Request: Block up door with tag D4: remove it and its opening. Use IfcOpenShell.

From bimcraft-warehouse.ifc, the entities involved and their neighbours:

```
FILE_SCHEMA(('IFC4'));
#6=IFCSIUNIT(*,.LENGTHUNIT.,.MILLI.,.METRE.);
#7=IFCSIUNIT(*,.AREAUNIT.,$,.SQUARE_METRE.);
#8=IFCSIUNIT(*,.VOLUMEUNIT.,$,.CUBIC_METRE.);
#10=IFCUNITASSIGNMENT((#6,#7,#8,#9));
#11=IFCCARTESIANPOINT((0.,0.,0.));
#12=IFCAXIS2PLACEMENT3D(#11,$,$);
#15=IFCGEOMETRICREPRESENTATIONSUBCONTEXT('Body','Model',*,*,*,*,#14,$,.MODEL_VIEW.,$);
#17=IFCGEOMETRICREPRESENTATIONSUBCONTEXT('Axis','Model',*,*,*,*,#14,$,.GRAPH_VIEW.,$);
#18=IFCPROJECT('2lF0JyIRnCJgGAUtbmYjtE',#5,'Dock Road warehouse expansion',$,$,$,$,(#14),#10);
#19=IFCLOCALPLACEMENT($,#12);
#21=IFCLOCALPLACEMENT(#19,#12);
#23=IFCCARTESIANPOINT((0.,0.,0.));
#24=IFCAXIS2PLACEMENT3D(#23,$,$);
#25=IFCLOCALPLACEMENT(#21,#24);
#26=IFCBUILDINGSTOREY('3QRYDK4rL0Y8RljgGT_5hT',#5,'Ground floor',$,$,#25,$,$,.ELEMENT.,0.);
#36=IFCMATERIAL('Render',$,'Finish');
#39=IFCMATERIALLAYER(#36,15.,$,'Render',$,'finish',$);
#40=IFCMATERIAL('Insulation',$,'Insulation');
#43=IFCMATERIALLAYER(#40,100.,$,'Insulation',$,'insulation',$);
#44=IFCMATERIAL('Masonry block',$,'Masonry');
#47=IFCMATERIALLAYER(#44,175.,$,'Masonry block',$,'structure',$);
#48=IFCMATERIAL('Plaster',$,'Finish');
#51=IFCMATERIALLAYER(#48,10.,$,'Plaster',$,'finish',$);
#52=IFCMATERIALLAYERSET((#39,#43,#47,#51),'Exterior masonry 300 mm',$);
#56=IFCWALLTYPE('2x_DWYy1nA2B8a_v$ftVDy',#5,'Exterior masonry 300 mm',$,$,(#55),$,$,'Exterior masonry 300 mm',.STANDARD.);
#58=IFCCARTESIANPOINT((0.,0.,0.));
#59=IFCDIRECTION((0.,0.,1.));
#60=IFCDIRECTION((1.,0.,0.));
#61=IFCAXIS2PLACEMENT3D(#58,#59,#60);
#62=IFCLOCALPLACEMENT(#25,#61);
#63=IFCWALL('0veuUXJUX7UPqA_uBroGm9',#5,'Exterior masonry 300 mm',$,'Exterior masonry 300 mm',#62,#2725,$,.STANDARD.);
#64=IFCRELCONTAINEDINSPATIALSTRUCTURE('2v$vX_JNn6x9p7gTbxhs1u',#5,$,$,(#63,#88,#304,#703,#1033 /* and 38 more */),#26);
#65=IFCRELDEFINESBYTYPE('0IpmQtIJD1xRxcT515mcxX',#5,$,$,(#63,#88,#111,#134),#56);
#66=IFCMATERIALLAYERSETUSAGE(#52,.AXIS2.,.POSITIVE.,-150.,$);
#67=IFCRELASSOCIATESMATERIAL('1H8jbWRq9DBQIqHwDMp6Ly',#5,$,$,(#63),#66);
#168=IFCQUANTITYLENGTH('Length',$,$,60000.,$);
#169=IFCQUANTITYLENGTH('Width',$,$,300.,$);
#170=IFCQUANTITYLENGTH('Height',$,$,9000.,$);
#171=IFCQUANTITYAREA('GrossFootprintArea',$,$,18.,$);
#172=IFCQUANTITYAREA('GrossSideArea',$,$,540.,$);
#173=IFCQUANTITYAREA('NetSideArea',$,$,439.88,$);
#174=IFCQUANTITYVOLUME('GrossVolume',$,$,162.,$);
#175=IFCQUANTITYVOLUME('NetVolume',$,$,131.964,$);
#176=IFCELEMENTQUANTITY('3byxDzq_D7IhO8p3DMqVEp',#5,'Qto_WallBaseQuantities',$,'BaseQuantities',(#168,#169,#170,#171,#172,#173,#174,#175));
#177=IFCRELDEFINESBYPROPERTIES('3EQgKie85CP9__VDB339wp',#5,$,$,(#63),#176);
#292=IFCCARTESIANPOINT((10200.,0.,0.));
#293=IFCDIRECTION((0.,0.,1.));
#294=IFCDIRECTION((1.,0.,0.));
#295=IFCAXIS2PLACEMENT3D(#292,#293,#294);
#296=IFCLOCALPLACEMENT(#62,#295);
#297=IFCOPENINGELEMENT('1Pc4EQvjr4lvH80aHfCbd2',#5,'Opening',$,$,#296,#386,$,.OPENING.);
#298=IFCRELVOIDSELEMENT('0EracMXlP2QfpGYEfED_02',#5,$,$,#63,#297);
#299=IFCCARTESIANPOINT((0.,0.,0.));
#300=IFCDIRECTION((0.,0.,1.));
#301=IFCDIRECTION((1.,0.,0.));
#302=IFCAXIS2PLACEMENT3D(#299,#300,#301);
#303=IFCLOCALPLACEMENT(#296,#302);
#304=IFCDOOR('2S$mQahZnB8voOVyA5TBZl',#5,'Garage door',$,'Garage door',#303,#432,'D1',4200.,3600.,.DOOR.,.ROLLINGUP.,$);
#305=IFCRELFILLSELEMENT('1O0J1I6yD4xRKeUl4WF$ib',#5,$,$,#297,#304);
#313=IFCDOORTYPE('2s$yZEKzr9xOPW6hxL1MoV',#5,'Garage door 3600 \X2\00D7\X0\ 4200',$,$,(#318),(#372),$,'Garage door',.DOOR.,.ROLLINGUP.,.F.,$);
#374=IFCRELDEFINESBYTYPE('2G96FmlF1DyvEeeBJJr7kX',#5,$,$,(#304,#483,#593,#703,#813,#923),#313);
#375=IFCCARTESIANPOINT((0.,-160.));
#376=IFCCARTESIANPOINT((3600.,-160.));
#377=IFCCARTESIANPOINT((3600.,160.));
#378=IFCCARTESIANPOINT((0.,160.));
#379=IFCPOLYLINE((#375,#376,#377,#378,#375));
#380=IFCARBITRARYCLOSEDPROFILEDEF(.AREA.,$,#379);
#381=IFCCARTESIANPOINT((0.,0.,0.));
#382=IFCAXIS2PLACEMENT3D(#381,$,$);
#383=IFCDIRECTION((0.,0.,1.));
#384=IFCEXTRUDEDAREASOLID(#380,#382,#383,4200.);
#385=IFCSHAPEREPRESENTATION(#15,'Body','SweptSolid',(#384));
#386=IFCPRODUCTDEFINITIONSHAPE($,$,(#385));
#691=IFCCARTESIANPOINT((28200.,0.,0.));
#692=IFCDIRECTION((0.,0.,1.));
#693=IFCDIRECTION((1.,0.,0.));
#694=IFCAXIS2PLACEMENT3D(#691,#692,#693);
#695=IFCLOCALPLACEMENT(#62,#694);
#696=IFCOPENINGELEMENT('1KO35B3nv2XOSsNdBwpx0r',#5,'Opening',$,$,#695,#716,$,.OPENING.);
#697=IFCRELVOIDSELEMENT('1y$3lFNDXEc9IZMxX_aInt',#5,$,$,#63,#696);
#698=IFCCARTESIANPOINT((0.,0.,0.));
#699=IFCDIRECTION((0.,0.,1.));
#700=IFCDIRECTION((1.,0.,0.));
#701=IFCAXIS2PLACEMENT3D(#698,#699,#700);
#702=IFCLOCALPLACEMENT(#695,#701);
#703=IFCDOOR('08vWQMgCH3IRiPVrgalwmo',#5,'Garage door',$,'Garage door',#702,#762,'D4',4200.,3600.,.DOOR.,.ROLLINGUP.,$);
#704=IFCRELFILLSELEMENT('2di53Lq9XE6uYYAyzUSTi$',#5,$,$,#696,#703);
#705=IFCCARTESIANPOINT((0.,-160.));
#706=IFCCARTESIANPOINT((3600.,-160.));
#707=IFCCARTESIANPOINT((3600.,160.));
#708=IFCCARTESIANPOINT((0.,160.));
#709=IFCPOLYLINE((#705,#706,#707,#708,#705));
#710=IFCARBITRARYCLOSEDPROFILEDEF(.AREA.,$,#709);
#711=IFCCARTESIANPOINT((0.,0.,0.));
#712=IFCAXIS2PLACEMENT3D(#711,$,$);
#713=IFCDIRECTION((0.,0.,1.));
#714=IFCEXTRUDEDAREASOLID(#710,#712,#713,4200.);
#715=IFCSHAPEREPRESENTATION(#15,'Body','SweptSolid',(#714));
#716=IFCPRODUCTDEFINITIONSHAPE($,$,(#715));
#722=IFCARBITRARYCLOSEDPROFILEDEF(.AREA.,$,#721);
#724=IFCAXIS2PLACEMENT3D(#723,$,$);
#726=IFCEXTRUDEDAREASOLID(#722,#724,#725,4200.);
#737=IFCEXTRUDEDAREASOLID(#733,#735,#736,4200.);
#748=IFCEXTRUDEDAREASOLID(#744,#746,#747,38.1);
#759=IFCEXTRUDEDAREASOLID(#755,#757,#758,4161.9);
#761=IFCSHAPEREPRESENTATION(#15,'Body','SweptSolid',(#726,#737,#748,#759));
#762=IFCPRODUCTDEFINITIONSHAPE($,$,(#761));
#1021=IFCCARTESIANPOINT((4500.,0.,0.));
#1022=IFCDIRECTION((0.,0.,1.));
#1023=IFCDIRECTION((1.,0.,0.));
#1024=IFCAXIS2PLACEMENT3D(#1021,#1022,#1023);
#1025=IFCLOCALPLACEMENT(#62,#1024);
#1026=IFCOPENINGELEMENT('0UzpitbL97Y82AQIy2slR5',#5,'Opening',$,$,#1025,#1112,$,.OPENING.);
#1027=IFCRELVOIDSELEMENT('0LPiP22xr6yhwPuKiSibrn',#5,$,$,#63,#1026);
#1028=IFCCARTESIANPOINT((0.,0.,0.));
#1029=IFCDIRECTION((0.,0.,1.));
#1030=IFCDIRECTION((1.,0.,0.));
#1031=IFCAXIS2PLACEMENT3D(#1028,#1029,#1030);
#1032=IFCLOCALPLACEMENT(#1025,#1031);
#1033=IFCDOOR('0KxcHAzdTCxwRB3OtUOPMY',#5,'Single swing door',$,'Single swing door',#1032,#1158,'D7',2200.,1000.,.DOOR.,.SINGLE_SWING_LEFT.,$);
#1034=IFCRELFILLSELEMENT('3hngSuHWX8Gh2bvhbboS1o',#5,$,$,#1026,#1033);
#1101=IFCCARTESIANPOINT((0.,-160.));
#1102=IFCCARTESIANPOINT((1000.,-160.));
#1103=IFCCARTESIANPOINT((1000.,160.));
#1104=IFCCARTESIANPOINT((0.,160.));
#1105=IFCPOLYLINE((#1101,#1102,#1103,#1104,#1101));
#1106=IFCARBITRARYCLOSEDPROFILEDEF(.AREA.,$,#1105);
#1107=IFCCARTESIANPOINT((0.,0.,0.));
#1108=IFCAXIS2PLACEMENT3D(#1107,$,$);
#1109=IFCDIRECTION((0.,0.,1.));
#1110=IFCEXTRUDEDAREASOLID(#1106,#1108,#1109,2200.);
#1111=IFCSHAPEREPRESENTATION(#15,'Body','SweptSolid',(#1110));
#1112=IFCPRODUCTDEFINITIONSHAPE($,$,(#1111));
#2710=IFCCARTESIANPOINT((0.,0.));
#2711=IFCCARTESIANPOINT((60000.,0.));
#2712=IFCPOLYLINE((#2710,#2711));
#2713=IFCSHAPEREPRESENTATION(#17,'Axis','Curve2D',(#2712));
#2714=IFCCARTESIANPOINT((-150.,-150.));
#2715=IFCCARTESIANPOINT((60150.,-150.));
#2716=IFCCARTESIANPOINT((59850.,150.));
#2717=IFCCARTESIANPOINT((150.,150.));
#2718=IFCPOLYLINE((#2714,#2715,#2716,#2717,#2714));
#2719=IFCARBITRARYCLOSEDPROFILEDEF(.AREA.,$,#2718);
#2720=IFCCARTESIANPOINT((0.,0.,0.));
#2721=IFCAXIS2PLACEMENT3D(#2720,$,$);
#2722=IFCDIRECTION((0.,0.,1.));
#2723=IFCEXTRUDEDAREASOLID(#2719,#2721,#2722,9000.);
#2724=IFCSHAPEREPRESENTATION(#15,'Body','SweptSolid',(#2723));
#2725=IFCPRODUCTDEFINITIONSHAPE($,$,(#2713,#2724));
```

```python
import ifcopenshell
import ifcopenshell.api.feature
import ifcopenshell.api.pset
import ifcopenshell.api.root
import ifcopenshell.geom
import ifcopenshell.util.element
import ifcopenshell.util.shape
import ifcopenshell.util.unit

model = ifcopenshell.open("bimcraft-warehouse.ifc")
area_scale = ifcopenshell.util.unit.calculate_unit_scale(model, "AREAUNIT")
volume_scale = ifcopenshell.util.unit.calculate_unit_scale(model, "VOLUMEUNIT")
settings = ifcopenshell.geom.settings()


def volume(element):
    """Net volume in cubic metres, openings subtracted."""
    shape = ifcopenshell.geom.create_shape(settings, element)
    return ifcopenshell.util.shape.get_volume(shape.geometry)


door = model.by_guid("08vWQMgCH3IRiPVrgalwmo")
opening = door.FillsVoids[0].RelatingOpeningElement
wall = opening.VoidsElements[0].RelatingBuildingElement
before = volume(wall)

ifcopenshell.api.root.remove_product(model, product=door)
ifcopenshell.api.feature.remove_feature(model, feature=opening)

after = volume(wall)
thickness = 0.3  # wall thickness in metres

# Update the wall's stored quantities.
qto = model.by_id(ifcopenshell.util.element.get_pset(wall, "Qto_WallBaseQuantities", should_inherit=False)["id"])
ifcopenshell.api.pset.edit_qto(model, qto=qto, properties={
    "NetSideArea": after / thickness / area_scale,
    "NetVolume": after / volume_scale,
})

print(f"wall volume {before:.3f} -> {after:.3f} m3")

model.write("bimcraft-warehouse_edited.ifc")
```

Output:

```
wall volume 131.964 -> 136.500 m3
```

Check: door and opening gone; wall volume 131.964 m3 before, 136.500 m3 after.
